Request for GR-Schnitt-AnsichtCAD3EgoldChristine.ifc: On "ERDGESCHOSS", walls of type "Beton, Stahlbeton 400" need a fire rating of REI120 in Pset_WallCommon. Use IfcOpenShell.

First a look at what the model holds.

```python
import ifcopenshell
import ifcopenshell.util.element

model = ifcopenshell.open("GR-Schnitt-AnsichtCAD3EgoldChristine.ifc")
print(model.schema)
storey = next(s for s in model.by_type("IfcBuildingStorey") if s.Name == "ERDGESCHOSS")
walls = [e for e in ifcopenshell.util.element.get_decomposition(storey) if e.is_a("IfcWall")]
seen = {}
for e in walls:
    element_type = ifcopenshell.util.element.get_type(e)
    key = (element_type.Name if element_type != e and element_type else None, ifcopenshell.util.element.get_pset(e, "Pset_WallCommon", "FireRating"))
    seen[key] = seen.get(key, 0) + 1
for (name, value), count in sorted(seen.items(), key=str):
    print(count, "x", name, "|", value)
```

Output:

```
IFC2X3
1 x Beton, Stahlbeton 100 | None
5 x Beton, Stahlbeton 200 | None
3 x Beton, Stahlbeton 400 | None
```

```python
import ifcopenshell
import ifcopenshell.api.pset
import ifcopenshell.util.element

model = ifcopenshell.open("GR-Schnitt-AnsichtCAD3EgoldChristine.ifc")

storey = next(s for s in model.by_type("IfcBuildingStorey") if s.Name == "ERDGESCHOSS")
walls = [e for e in ifcopenshell.util.element.get_decomposition(storey) if e.is_a("IfcWall")]

count = 0
for e in walls:
    element_type = ifcopenshell.util.element.get_type(e)
    if element_type in (None, e) or element_type.Name != "Beton, Stahlbeton 400":
        continue
    # add_pset returns the element's existing set when there is one.
    pset = ifcopenshell.api.pset.add_pset(model, product=e, name="Pset_WallCommon")
    ifcopenshell.api.pset.edit_pset(model, pset=pset, properties={"FireRating": "REI120"})
    count += 1

print(count, "walls updated")

model.write("GR-Schnitt-AnsichtCAD3EgoldChristine-out.ifc")
```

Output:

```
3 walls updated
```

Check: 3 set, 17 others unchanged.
